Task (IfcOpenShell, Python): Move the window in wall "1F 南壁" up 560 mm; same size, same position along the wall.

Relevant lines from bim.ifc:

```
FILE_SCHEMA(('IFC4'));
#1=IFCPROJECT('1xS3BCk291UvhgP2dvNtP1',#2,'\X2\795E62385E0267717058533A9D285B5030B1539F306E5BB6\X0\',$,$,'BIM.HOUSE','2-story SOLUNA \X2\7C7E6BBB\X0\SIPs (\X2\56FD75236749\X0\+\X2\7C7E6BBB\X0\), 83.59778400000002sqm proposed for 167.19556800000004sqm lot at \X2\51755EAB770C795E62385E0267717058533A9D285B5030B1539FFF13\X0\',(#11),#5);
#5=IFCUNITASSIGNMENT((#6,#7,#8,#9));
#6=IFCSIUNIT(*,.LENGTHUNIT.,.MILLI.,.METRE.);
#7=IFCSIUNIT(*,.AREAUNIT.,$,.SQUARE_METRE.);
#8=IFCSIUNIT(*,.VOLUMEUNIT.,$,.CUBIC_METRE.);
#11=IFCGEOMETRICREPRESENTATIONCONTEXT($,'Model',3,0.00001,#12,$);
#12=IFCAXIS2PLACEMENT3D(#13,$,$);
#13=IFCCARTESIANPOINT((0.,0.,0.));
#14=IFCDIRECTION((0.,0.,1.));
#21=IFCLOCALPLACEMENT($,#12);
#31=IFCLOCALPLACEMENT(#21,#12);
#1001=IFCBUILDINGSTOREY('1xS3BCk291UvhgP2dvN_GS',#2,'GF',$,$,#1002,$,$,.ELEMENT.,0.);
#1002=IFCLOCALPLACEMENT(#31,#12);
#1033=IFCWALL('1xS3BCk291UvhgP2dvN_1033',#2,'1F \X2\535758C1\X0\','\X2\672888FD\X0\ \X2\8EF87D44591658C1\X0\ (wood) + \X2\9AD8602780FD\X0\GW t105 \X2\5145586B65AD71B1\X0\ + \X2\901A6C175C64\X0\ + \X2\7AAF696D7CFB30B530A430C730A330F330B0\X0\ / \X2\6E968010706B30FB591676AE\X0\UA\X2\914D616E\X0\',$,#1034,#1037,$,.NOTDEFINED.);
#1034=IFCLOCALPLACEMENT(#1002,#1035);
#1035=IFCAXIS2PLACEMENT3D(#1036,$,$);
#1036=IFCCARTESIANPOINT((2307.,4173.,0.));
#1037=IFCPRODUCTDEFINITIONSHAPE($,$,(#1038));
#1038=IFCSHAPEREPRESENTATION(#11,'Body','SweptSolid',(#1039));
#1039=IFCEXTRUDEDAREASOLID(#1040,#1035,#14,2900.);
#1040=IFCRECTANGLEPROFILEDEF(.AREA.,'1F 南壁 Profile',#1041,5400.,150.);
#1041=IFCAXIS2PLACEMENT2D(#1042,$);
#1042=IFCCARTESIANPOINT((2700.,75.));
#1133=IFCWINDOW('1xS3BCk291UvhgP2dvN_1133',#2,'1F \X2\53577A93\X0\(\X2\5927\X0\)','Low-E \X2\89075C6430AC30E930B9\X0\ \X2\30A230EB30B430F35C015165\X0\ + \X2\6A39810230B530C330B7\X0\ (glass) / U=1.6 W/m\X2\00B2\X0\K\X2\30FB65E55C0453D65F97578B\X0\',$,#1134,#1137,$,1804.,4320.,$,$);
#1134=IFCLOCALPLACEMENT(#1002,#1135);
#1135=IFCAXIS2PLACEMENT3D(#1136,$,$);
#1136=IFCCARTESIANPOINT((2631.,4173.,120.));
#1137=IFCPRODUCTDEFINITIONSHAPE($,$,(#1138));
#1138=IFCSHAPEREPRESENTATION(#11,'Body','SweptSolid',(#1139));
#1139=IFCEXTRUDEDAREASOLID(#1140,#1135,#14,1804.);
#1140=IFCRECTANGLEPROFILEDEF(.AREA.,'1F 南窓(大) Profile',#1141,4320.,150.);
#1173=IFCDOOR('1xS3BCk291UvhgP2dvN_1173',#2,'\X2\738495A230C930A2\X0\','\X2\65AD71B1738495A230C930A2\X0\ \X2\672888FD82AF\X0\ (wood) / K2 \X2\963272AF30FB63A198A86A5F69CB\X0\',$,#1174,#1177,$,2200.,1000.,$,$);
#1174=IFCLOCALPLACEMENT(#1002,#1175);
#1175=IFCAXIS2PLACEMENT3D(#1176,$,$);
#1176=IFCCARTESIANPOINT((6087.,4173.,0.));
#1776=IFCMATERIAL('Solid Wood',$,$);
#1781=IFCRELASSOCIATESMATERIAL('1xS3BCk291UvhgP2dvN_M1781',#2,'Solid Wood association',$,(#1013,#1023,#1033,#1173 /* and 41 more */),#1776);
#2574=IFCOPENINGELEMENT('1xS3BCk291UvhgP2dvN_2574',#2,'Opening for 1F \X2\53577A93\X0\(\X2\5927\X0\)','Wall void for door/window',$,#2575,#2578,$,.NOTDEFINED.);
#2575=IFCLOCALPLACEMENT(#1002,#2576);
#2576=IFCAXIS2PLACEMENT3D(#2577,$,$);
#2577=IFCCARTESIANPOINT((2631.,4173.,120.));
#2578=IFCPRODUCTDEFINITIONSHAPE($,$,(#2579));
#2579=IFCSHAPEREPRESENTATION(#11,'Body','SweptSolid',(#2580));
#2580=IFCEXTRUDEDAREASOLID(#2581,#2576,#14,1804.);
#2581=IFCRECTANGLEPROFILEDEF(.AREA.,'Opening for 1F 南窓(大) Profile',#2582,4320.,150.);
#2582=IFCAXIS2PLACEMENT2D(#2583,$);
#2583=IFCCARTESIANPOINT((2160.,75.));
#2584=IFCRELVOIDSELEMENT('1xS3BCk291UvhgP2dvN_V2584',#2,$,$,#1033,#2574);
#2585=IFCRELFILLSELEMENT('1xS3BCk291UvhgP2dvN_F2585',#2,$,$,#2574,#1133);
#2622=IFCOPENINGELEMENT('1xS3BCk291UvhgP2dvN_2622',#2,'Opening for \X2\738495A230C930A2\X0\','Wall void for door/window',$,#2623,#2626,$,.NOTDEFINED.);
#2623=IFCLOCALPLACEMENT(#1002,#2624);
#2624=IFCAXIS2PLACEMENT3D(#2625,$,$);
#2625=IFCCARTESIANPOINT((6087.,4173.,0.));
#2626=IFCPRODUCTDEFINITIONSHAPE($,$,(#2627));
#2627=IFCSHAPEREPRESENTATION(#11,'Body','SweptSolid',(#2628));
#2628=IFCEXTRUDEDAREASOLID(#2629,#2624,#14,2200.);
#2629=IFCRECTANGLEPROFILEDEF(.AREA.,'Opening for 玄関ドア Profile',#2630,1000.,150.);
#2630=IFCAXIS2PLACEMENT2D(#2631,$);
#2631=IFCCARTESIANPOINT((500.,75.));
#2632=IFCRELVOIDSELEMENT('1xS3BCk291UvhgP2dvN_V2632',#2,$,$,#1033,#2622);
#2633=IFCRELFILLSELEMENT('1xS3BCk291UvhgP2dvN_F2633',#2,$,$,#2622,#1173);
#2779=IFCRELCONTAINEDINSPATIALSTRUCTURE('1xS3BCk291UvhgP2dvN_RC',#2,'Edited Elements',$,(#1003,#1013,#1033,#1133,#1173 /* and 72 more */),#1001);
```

```python
import numpy as np
import ifcopenshell
import ifcopenshell.api.geometry
import ifcopenshell.util.placement
import ifcopenshell.util.unit

model = ifcopenshell.open("bim.ifc")
unit_scale = ifcopenshell.util.unit.calculate_unit_scale(model)

window = model.by_guid("1xS3BCk291UvhgP2dvN_1133")
opening = window.FillsVoids[0].RelatingOpeningElement
dz = 0.56 / unit_scale

shift = np.array([0.0, 0.0, dz])
# The window is not placed relative to its opening, so move both.
for product in (opening, window):
    matrix = ifcopenshell.util.placement.get_local_placement(product.ObjectPlacement)
    matrix[:3, 3] += shift
    ifcopenshell.api.geometry.edit_object_placement(model, product=product, matrix=matrix, is_si=False)

print(f"moved by {dz * unit_scale:+.3f} m")

model.write("bim_rev.ifc")
```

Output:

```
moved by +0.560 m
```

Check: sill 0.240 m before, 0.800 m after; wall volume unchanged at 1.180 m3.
